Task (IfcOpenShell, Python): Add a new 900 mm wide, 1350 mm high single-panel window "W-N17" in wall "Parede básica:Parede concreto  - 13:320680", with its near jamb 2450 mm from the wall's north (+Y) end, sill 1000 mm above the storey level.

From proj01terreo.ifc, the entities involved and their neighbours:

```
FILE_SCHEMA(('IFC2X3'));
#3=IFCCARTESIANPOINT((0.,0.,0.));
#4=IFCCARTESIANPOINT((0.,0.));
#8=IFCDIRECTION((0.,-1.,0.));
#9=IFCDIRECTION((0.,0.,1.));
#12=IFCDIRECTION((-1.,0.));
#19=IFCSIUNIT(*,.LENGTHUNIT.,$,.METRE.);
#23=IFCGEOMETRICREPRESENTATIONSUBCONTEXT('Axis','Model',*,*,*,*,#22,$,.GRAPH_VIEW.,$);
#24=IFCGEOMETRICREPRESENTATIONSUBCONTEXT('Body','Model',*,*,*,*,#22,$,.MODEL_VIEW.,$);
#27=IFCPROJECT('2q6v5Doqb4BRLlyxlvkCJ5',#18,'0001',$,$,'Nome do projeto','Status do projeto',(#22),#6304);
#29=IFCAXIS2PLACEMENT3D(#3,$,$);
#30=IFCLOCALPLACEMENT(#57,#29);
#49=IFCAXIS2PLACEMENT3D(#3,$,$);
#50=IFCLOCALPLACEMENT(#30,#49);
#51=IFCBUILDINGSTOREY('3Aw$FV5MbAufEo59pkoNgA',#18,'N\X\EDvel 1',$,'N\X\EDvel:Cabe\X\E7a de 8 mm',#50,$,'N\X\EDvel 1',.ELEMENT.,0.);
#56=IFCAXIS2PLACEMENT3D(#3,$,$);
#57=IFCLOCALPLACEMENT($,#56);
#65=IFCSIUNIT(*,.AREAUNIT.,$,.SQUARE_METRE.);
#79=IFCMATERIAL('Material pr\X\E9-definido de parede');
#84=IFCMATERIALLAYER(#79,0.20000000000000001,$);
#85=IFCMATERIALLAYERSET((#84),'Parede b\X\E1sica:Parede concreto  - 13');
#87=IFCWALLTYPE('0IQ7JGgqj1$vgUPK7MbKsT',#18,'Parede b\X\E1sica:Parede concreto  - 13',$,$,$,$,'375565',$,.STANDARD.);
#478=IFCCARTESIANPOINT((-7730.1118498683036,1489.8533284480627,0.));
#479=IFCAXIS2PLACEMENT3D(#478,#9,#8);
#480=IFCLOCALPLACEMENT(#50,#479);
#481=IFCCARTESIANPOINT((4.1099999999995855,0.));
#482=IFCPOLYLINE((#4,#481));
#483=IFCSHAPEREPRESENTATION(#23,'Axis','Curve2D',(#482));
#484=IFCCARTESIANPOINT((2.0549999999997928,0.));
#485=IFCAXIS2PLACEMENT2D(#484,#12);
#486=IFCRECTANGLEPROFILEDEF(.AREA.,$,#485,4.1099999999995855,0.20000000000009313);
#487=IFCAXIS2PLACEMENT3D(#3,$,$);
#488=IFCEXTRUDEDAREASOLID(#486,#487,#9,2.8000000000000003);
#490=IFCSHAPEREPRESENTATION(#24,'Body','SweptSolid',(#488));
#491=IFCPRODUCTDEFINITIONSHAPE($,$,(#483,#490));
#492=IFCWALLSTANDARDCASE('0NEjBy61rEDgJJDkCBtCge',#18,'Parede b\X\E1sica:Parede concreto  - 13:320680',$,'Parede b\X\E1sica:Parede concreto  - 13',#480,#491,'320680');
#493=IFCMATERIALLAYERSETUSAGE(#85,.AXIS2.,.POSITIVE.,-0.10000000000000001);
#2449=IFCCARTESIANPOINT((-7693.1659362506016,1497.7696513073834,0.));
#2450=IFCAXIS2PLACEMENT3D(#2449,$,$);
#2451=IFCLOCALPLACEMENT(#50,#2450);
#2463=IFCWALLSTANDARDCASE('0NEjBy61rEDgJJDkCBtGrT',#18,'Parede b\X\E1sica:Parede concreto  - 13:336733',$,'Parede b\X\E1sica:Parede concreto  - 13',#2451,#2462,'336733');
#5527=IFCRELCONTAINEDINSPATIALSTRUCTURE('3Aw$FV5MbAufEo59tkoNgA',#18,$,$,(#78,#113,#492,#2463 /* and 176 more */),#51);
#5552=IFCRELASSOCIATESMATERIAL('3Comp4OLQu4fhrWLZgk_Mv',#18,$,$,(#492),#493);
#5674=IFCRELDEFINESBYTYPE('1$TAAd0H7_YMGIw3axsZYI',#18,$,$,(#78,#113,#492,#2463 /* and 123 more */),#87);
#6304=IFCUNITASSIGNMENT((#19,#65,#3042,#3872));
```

```python
import numpy as np
import ifcopenshell
import ifcopenshell.api.feature
import ifcopenshell.api.geometry
import ifcopenshell.api.root
import ifcopenshell.api.spatial
import ifcopenshell.api.type
import ifcopenshell.geom
import ifcopenshell.util.element
import ifcopenshell.util.placement
import ifcopenshell.util.representation
import ifcopenshell.util.shape
import ifcopenshell.util.unit

model = ifcopenshell.open("proj01terreo.ifc")
unit_scale = ifcopenshell.util.unit.calculate_unit_scale(model)
settings = ifcopenshell.geom.settings()


def volume(element):
    """Net volume in cubic metres, openings subtracted."""
    shape = ifcopenshell.geom.create_shape(settings, element)
    return ifcopenshell.util.shape.get_volume(shape.geometry)


wall = model.by_guid("0NEjBy61rEDgJJDkCBtCge")
storey = ifcopenshell.util.element.get_container(wall, ifc_class="IfcBuildingStorey")
context = ifcopenshell.util.representation.get_context(model, "Model", "Body", "MODEL_VIEW")
before = volume(wall)

width, height, from_end, sill = 0.9, 1.35, 2.45, 1  # metres

# The wall runs along its own X axis, and the end named is its -X end.
wall_shape = ifcopenshell.geom.create_shape(settings, wall)
x, y, z = ifcopenshell.util.shape.get_vertices(wall_shape.geometry).T
start = x.min() + from_end
face, thickness = float(y.min()), float(y.max() - y.min())
wall_matrix = ifcopenshell.util.placement.get_local_placement(wall.ObjectPlacement)
level = ifcopenshell.util.placement.get_local_placement(storey.ObjectPlacement)[2, 3]


def in_wall(x, y):
    """Placement at x, y metres in the wall's axes, at sill height."""
    matrix = wall_matrix.copy()
    matrix[:, 3] = wall_matrix @ np.array([x / unit_scale, y / unit_scale, 0.0, 1.0])
    matrix[2, 3] = level + sill / unit_scale
    return matrix


# Opening: a box that overshoots both wall faces by 50 mm.
opening = ifcopenshell.api.root.create_entity(model, ifc_class="IfcOpeningElement")
box = ifcopenshell.api.geometry.add_wall_representation(
    model, context=context, length=width, height=height, thickness=thickness + 0.1
)
ifcopenshell.api.geometry.assign_representation(model, product=opening, representation=box)
ifcopenshell.api.geometry.edit_object_placement(model, product=opening, matrix=in_wall(start, face - 0.05), is_si=False)
ifcopenshell.api.feature.add_feature(model, feature=opening, element=wall)

window = ifcopenshell.api.root.create_entity(model, ifc_class="IfcWindow", name="W-N17")
window.OverallWidth, window.OverallHeight = width / unit_scale, height / unit_scale
body = ifcopenshell.api.geometry.add_window_representation(
    model,
    context=context,
    overall_width=window.OverallWidth,
    overall_height=window.OverallHeight,
    partition_type="SINGLE_PANEL",
)
ifcopenshell.api.geometry.assign_representation(model, product=window, representation=body)
ifcopenshell.api.spatial.assign_container(model, products=[window], relating_structure=storey)
fills = ifcopenshell.api.feature.add_filling(model, opening=opening, element=window)
fills.OwnerHistory = window.OwnerHistory  # required in IFC2X3

# IFC2X3 keeps the operation on the window style.
style = ifcopenshell.api.root.create_entity(model, ifc_class="IfcWindowStyle", name="W-N17")
style.OperationType, style.ConstructionType = "SINGLE_PANEL", "NOTDEFINED"
style.ParameterTakesPrecedence = style.Sizeable = False
ifcopenshell.api.type.assign_type(model, related_objects=[window], relating_type=style)

# Centre the window in the wall's thickness.
ifcopenshell.api.geometry.edit_object_placement(model, product=window, matrix=in_wall(start, face), is_si=False)
window_shape = ifcopenshell.geom.create_shape(settings, window)
depth = ifcopenshell.util.shape.get_vertices(window_shape.geometry)[:, 1]
offset = face + thickness / 2 - (depth.min() + depth.max()) / 2
ifcopenshell.api.geometry.edit_object_placement(model, product=window, matrix=in_wall(start, offset), is_si=False)

after = volume(wall)

print(f"wall volume {before:.3f} -> {after:.3f} m3")

model.write("proj01terreo_updated.ifc")
```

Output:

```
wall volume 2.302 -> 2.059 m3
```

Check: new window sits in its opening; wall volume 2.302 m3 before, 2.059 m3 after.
